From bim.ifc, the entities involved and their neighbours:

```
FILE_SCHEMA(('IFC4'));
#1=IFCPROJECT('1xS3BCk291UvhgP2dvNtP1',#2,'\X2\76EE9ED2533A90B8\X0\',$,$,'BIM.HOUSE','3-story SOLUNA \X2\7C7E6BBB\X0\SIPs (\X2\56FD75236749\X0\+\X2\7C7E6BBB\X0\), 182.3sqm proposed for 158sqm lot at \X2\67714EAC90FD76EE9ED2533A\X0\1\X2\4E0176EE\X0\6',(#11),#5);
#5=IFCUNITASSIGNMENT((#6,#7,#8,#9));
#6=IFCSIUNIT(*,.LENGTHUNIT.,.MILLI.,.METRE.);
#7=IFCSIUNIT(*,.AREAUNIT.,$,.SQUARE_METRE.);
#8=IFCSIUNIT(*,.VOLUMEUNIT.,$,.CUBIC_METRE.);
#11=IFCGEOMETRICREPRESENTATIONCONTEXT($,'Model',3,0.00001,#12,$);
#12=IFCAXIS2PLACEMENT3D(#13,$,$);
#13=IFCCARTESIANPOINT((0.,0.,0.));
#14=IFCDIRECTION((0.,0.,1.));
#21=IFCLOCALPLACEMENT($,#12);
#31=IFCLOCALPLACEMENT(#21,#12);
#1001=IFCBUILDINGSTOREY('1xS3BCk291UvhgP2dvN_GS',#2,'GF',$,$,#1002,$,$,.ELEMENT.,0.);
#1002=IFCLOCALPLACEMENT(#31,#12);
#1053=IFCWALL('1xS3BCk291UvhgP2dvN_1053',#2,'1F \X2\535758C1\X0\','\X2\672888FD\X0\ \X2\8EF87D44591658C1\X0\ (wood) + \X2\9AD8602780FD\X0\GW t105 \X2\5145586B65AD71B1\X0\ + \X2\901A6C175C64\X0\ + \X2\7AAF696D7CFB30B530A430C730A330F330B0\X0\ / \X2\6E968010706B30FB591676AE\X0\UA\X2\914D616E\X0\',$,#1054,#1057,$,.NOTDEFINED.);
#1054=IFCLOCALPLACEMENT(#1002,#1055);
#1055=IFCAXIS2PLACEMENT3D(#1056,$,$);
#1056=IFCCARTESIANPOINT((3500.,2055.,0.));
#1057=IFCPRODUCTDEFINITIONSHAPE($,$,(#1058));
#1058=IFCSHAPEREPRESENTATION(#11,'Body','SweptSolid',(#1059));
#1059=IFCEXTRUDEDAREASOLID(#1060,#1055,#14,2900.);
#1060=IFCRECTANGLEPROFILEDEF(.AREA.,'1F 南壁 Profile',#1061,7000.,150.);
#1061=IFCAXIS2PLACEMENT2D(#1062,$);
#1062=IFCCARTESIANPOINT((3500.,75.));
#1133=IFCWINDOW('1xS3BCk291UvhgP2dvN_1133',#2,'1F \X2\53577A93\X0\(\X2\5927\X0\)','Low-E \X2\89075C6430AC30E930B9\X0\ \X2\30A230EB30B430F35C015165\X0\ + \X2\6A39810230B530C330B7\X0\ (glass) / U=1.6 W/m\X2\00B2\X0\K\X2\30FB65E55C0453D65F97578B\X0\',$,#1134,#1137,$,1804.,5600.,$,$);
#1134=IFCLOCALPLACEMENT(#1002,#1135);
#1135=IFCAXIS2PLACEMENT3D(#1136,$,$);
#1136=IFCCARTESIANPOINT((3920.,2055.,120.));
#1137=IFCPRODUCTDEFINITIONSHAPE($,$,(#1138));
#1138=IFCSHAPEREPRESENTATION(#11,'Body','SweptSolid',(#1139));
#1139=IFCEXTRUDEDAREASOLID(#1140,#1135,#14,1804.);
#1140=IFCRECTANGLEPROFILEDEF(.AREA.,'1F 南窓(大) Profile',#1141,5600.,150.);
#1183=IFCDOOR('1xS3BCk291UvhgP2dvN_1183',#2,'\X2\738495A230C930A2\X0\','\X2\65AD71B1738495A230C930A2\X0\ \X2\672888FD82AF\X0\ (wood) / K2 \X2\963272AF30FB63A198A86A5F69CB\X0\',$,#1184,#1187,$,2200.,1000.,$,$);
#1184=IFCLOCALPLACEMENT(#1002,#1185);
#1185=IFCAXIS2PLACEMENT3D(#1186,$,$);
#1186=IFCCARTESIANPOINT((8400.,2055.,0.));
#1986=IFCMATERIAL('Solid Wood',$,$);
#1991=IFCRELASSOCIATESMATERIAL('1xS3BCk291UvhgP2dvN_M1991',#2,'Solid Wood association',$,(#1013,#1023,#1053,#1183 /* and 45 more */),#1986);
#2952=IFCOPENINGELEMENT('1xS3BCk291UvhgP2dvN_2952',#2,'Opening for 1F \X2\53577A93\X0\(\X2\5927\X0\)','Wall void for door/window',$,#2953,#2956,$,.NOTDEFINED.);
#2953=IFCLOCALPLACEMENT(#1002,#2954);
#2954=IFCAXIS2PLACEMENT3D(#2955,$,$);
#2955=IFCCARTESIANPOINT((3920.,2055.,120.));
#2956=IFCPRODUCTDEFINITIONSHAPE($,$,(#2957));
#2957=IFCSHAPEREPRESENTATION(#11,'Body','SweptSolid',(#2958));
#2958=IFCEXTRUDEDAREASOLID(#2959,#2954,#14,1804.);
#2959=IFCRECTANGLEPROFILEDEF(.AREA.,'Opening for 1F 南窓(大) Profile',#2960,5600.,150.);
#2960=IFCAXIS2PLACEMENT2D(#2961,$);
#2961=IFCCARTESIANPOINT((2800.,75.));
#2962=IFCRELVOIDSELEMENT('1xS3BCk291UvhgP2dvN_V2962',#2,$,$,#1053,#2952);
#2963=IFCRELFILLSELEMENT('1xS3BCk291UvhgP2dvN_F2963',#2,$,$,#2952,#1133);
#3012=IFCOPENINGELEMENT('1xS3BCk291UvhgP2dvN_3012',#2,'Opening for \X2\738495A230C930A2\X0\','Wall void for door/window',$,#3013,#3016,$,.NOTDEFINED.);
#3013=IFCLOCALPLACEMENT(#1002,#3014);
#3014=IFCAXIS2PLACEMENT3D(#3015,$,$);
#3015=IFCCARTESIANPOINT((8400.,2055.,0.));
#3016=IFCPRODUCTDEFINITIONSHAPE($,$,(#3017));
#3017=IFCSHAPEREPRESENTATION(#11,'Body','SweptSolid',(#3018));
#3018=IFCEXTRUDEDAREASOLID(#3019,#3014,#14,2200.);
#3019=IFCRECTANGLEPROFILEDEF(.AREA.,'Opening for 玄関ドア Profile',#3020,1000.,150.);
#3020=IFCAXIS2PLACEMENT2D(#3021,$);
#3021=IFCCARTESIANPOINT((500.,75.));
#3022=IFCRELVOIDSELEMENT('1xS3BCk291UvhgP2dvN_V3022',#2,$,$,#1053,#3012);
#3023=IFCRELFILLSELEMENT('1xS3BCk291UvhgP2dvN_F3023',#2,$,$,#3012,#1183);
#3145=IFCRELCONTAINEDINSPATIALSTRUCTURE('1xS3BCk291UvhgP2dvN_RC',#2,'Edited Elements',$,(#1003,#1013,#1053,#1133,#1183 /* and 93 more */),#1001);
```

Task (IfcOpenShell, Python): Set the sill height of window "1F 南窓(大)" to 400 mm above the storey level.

```python
import numpy as np
import ifcopenshell
import ifcopenshell.api.geometry
import ifcopenshell.geom
import ifcopenshell.util.element
import ifcopenshell.util.placement
import ifcopenshell.util.shape
import ifcopenshell.util.unit

model = ifcopenshell.open("bim.ifc")
unit_scale = ifcopenshell.util.unit.calculate_unit_scale(model)

window = model.by_guid("1xS3BCk291UvhgP2dvN_1133")
opening = window.FillsVoids[0].RelatingOpeningElement
storey = ifcopenshell.util.element.get_container(window, ifc_class="IfcBuildingStorey")
level = ifcopenshell.util.placement.get_local_placement(storey.ObjectPlacement)[2, 3]

# The opening's origin need not be at the sill, so measure its lowest point.
shape = ifcopenshell.geom.create_shape(ifcopenshell.geom.settings(), opening)
bottom = ifcopenshell.util.shape.get_shape_bottom_elevation(shape, shape.geometry) / unit_scale
dz = level + 0.4 / unit_scale - bottom

shift = np.array([0.0, 0.0, dz])
# The window is not placed relative to its opening, so move both.
for product in (opening, window):
    matrix = ifcopenshell.util.placement.get_local_placement(product.ObjectPlacement)
    matrix[:3, 3] += shift
    ifcopenshell.api.geometry.edit_object_placement(model, product=product, matrix=matrix, is_si=False)

print(f"moved by {dz * unit_scale:+.3f} m")

model.write("bim_rev.ifc")
```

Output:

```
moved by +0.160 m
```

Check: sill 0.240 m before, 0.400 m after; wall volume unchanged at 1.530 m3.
